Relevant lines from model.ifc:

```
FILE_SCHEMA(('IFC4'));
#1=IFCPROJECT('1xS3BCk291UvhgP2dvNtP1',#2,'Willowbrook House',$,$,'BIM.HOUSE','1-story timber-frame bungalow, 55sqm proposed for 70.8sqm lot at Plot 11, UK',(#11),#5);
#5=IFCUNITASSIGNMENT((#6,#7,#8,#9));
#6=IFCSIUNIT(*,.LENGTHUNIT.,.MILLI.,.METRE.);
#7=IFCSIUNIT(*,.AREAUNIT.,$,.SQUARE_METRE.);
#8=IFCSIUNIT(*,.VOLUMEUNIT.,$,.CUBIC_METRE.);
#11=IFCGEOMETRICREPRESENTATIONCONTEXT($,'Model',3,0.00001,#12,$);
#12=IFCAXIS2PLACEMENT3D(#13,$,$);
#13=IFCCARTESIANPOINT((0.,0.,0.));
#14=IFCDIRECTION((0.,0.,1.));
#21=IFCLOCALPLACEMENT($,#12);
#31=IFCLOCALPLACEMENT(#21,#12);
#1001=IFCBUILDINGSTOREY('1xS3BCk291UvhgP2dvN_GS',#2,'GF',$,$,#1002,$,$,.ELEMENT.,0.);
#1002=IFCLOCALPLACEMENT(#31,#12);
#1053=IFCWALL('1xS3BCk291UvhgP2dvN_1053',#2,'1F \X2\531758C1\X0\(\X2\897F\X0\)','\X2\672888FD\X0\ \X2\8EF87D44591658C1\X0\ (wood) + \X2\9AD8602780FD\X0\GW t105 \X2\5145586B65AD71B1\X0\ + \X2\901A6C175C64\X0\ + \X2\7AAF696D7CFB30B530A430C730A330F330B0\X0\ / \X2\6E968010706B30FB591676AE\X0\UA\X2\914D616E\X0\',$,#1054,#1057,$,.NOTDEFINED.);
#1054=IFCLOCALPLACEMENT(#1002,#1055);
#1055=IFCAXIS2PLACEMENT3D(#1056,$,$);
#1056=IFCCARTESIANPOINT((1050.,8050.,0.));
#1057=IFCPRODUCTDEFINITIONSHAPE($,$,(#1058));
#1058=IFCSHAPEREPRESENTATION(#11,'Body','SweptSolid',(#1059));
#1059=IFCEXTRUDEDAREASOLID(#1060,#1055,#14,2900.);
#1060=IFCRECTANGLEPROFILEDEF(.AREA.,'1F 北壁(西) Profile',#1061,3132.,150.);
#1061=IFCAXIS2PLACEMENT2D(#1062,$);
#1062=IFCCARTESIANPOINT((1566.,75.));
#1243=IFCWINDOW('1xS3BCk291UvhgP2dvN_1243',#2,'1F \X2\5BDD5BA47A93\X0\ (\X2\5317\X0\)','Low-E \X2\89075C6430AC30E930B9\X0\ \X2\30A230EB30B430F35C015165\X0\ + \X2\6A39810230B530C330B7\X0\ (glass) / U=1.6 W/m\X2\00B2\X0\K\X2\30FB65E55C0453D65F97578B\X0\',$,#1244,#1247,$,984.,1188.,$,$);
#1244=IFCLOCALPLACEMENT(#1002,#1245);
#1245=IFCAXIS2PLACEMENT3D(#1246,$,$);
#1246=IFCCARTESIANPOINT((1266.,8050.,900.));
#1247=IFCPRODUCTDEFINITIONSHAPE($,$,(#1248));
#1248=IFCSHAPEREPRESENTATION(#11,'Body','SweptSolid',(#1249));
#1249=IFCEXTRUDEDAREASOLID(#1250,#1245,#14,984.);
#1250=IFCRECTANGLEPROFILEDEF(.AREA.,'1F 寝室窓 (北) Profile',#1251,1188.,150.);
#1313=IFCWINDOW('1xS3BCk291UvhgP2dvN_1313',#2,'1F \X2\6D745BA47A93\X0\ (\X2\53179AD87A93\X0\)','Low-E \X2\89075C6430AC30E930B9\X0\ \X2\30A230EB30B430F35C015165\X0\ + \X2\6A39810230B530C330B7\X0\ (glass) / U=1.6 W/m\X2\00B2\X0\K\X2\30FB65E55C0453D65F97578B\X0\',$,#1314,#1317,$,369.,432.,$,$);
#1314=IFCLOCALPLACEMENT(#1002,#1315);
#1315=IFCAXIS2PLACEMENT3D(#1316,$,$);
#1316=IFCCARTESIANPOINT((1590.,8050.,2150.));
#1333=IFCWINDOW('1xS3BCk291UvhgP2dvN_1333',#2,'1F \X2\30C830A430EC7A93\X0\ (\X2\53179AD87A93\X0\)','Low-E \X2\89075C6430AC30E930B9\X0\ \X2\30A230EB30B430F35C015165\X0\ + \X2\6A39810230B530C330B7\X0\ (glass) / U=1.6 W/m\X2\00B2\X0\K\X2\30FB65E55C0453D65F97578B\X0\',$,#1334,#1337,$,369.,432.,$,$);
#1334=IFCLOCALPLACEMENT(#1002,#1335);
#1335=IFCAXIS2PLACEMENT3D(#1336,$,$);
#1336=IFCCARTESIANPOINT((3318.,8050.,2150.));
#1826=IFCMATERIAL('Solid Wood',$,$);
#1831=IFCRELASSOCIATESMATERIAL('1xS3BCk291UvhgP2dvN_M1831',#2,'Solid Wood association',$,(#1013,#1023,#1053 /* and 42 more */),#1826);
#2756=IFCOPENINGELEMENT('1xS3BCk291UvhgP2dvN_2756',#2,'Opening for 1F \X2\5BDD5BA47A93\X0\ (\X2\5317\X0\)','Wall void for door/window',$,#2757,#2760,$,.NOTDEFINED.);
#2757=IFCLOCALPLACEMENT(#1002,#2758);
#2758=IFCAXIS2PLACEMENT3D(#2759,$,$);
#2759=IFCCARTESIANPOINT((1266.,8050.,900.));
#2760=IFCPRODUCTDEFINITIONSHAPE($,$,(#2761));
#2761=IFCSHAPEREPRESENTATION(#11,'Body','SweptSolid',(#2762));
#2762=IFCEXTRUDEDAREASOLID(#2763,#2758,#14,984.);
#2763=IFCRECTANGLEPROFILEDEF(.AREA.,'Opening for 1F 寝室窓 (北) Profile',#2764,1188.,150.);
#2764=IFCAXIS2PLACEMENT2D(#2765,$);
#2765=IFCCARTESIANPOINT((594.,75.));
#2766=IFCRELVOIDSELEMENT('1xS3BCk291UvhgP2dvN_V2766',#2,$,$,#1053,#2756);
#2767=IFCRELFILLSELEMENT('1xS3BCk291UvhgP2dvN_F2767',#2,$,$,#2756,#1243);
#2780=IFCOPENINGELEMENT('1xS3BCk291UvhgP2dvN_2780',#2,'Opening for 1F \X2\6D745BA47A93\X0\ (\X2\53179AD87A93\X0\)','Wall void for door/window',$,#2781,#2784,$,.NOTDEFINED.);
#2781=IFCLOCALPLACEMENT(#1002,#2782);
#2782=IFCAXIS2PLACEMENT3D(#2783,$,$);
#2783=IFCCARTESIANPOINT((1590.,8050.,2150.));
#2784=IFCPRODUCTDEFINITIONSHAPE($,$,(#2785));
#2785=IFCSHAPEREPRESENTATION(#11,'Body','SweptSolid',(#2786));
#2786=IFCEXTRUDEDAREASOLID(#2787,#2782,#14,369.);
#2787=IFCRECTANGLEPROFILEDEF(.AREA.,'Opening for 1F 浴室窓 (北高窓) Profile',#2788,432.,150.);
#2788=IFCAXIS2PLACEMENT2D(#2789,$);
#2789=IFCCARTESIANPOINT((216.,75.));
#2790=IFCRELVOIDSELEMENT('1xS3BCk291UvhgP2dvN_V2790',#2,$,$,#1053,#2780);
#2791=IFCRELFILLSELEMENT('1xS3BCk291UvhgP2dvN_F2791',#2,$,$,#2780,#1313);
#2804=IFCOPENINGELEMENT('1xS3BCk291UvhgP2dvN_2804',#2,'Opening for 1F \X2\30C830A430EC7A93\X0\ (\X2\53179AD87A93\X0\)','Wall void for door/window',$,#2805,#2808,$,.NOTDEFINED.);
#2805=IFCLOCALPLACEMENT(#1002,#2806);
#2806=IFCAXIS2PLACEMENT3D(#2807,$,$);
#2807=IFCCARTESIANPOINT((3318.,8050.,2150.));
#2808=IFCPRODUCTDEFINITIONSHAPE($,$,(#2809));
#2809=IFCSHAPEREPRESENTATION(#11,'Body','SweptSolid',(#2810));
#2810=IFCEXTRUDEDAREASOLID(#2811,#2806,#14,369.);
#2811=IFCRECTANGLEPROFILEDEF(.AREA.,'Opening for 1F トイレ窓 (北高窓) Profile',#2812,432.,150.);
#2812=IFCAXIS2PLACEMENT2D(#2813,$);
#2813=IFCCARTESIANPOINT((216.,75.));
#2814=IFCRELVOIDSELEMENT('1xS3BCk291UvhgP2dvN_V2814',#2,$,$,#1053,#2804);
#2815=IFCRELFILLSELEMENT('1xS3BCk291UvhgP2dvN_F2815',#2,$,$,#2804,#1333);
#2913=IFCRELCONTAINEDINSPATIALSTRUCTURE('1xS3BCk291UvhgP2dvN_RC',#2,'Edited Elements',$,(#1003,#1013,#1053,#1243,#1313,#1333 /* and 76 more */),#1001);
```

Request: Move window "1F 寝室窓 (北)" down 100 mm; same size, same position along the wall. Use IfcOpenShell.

```python
import numpy as np
import ifcopenshell
import ifcopenshell.api.geometry
import ifcopenshell.util.placement
import ifcopenshell.util.unit

model = ifcopenshell.open("model.ifc")
unit_scale = ifcopenshell.util.unit.calculate_unit_scale(model)

window = model.by_id(1243)
opening = window.FillsVoids[0].RelatingOpeningElement
dz = -0.1 / unit_scale

shift = np.array([0.0, 0.0, dz])
# The window is not placed relative to its opening, so move both.
for product in (opening, window):
    matrix = ifcopenshell.util.placement.get_local_placement(product.ObjectPlacement)
    matrix[:3, 3] += shift
    ifcopenshell.api.geometry.edit_object_placement(model, product=product, matrix=matrix, is_si=False)

print(f"moved by {dz * unit_scale:+.3f} m")

model.write("model_updated.ifc")
```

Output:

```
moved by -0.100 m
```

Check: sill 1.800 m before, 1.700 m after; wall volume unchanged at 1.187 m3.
